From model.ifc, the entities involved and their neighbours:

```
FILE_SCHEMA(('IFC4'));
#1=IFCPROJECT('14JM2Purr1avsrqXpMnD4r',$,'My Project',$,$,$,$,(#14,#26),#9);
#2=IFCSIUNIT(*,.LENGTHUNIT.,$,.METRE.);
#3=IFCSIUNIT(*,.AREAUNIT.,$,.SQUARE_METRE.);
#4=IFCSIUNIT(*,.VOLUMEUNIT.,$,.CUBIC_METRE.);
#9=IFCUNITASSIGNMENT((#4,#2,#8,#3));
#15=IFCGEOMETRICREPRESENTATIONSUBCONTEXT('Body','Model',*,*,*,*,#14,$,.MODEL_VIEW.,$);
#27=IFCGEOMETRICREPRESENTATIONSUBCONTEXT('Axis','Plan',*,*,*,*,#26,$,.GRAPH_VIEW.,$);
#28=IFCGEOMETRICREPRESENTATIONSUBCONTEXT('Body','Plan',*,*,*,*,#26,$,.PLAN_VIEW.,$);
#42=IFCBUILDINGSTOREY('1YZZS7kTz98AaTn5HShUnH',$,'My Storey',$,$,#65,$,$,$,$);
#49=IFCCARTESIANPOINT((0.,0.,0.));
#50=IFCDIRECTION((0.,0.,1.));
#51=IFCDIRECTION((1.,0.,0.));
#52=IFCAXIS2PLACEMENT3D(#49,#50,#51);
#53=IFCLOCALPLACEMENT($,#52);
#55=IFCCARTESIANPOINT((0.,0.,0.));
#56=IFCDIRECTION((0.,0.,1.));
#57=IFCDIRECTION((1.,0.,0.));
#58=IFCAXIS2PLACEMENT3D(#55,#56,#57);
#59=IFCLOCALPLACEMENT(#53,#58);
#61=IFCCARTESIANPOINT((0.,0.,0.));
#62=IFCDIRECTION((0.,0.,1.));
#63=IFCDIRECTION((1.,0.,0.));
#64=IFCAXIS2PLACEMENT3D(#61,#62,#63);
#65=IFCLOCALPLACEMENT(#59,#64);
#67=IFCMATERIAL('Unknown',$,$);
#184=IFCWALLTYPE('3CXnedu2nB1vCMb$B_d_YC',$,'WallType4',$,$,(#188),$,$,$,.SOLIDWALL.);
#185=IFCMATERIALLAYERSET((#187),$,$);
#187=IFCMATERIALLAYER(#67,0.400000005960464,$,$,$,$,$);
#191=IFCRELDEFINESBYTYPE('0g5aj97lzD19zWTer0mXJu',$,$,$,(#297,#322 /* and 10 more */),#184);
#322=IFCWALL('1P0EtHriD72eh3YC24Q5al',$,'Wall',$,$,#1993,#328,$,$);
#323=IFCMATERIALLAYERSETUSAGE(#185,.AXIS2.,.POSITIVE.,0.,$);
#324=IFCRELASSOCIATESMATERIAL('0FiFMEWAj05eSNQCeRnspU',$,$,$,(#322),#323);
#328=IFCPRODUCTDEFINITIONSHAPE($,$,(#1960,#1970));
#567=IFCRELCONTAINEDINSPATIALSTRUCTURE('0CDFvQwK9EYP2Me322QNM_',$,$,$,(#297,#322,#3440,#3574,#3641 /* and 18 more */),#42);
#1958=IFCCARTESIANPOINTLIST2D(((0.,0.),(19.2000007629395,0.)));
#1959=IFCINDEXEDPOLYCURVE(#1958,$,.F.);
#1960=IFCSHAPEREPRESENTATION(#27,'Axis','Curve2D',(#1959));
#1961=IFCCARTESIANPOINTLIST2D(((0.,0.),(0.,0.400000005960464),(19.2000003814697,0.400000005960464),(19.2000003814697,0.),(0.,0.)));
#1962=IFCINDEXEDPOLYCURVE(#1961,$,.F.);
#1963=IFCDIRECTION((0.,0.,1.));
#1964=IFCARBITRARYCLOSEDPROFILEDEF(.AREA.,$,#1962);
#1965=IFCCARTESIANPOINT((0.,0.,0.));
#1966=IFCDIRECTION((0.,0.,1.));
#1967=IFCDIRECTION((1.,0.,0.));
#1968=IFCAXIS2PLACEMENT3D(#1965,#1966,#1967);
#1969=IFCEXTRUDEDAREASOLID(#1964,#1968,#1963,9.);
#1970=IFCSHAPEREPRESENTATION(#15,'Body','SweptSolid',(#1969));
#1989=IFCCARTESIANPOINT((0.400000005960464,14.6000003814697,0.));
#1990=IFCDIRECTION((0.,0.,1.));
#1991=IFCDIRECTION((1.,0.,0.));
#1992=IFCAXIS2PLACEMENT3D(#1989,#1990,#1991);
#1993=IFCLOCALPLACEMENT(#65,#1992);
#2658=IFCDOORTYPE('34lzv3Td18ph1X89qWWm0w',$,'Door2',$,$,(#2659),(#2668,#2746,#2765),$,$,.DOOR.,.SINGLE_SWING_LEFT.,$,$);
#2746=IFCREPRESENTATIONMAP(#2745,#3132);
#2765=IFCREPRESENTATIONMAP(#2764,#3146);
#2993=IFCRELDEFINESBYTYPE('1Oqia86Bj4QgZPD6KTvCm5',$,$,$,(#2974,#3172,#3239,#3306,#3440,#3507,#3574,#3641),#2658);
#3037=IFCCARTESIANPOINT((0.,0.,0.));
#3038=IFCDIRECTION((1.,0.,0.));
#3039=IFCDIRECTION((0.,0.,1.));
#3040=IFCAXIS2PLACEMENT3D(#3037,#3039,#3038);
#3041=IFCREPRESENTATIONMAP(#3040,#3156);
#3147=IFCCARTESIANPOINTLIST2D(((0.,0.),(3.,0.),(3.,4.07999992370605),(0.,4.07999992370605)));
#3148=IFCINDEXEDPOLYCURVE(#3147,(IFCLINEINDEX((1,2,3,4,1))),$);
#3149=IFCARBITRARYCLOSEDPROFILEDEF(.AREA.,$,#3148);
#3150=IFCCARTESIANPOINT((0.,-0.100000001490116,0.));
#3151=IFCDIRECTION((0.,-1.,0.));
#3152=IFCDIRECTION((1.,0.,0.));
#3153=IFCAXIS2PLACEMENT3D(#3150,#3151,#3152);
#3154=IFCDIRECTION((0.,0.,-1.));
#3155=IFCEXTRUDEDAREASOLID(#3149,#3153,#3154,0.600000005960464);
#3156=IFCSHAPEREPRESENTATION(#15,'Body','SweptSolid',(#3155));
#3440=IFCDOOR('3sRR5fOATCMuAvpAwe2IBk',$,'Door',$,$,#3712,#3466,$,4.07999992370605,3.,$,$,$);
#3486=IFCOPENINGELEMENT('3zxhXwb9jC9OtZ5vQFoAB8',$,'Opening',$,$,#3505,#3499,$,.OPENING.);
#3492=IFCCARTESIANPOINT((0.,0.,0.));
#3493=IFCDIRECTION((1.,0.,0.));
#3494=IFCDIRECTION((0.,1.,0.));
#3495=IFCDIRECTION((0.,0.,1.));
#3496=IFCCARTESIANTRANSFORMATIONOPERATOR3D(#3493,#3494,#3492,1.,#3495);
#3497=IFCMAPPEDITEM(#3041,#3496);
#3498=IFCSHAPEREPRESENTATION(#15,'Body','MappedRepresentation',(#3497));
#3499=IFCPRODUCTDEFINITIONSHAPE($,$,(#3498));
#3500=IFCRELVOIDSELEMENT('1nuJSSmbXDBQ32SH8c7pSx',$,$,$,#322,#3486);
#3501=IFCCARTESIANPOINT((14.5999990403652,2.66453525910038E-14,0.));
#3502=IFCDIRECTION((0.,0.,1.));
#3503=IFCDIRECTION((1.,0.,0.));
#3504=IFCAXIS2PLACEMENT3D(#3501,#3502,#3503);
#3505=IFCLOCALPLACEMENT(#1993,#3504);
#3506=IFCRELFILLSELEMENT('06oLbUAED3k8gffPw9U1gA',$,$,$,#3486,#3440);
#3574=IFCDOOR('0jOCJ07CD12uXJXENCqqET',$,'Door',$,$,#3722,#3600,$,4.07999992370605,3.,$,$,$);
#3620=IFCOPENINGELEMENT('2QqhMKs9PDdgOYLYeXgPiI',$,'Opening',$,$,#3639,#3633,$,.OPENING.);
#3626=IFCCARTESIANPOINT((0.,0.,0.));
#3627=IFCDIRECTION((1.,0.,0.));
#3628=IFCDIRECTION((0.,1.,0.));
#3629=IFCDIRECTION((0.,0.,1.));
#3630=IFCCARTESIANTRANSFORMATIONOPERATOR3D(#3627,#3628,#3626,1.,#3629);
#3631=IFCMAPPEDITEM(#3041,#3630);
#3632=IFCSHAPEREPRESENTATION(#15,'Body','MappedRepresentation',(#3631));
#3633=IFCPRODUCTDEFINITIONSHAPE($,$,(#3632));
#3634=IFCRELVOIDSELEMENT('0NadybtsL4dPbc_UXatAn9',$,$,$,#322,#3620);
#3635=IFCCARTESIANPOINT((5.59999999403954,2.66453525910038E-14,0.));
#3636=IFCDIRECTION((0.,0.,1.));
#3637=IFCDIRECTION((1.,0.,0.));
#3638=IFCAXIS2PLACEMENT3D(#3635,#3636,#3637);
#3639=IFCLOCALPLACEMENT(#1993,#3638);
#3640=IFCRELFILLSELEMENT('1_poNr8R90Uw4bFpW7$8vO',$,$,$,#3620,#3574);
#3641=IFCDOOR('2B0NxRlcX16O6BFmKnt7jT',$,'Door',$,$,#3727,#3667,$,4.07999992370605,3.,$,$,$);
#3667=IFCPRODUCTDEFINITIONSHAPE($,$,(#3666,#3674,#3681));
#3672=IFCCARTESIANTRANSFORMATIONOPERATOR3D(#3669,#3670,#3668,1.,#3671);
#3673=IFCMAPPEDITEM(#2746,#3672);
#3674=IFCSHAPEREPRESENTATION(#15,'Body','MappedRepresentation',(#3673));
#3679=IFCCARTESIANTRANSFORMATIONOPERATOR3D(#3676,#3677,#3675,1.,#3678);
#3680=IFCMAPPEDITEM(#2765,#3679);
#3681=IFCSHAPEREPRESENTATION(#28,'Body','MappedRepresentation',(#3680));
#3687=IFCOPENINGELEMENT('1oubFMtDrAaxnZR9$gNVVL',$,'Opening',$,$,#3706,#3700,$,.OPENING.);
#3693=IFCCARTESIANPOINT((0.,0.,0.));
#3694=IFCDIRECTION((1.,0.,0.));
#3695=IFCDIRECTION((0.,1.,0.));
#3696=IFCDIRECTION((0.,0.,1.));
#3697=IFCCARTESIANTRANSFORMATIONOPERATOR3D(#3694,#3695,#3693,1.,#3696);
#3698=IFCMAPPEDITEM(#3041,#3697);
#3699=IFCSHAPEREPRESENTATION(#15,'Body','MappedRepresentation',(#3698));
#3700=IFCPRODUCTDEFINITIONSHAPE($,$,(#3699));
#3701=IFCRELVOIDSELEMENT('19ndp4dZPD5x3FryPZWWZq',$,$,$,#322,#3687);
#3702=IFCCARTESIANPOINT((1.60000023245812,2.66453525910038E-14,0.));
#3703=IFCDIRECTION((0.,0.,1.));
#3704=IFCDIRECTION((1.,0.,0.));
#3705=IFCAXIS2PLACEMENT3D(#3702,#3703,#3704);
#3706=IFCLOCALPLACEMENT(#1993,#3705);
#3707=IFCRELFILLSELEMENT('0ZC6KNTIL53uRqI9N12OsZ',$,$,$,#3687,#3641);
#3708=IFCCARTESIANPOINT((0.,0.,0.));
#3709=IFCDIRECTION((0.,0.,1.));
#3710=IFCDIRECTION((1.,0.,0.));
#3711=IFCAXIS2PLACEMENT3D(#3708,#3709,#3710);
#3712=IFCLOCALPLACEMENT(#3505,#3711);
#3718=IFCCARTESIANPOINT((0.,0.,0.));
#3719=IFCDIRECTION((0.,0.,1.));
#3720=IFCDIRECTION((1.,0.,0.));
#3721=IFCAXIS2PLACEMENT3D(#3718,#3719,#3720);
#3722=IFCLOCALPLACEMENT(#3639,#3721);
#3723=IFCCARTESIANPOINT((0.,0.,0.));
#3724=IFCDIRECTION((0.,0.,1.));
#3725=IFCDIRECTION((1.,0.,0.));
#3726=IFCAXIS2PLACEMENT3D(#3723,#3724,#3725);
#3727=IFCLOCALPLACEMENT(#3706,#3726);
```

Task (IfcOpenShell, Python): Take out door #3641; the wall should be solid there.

```python
import ifcopenshell
import ifcopenshell.api.feature
import ifcopenshell.api.root
import ifcopenshell.geom
import ifcopenshell.util.shape

model = ifcopenshell.open("model.ifc")
settings = ifcopenshell.geom.settings()


def volume(element):
    """Net volume in cubic metres, openings subtracted."""
    shape = ifcopenshell.geom.create_shape(settings, element)
    return ifcopenshell.util.shape.get_volume(shape.geometry)


door = model.by_id(3641)
opening = door.FillsVoids[0].RelatingOpeningElement
wall = opening.VoidsElements[0].RelatingBuildingElement
before = volume(wall)

ifcopenshell.api.root.remove_product(model, product=door)
ifcopenshell.api.feature.remove_feature(model, feature=opening)

after = volume(wall)

print(f"wall volume {before:.3f} -> {after:.3f} m3")

model.write("model-out.ifc")
```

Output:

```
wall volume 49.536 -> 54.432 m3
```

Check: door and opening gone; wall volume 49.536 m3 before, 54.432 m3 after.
